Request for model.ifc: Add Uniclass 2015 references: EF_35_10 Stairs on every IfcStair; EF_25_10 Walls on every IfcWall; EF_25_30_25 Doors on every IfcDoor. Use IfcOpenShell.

First a look at what the model holds.

```python
import ifcopenshell

model = ifcopenshell.open("model.ifc")
print(model.schema)
print("classifications:", [c.Name for c in model.by_type("IfcClassification")])
for ifc_class in ("IfcDoor", "IfcRoof", "IfcStair", "IfcWall", "IfcWindow"):
    print(ifc_class, len(model.by_type(ifc_class)))
```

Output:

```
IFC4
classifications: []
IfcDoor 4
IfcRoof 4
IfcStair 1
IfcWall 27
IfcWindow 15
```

```python
import ifcopenshell
import ifcopenshell.api.classification

model = ifcopenshell.open("model.ifc")

system = ifcopenshell.api.classification.add_classification(model, classification="Uniclass 2015")

codes = {
    "IfcStair": ("EF_35_10", "Stairs"),
    "IfcWall": ("EF_25_10", "Walls"),
    "IfcDoor": ("EF_25_30_25", "Doors"),
}
for ifc_class, (code, name) in codes.items():
    products = model.by_type(ifc_class)
    ifcopenshell.api.classification.add_reference(
        model, products=products, classification=system, identification=code, name=name
    )
    print(code, len(products))

model.write("model_rev.ifc")
```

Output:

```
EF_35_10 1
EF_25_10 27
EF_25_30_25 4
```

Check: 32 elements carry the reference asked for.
